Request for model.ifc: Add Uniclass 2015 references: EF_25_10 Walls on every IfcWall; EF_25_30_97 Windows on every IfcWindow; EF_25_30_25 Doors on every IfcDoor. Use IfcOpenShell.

First a look at what the model holds.

```python
import ifcopenshell

model = ifcopenshell.open("model.ifc")
print(model.schema)
print("classifications:", [c.Name for c in model.by_type("IfcClassification")])
for ifc_class in ("IfcDoor", "IfcRoof", "IfcStair", "IfcWall", "IfcWindow"):
    print(ifc_class, len(model.by_type(ifc_class)))
```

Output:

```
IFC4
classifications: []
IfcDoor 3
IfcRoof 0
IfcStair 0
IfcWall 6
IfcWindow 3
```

```python
import ifcopenshell
import ifcopenshell.api.classification

model = ifcopenshell.open("model.ifc")

system = ifcopenshell.api.classification.add_classification(model, classification="Uniclass 2015")

codes = {
    "IfcWall": ("EF_25_10", "Walls"),
    "IfcWindow": ("EF_25_30_97", "Windows"),
    "IfcDoor": ("EF_25_30_25", "Doors"),
}
for ifc_class, (code, name) in codes.items():
    products = model.by_type(ifc_class)
    ifcopenshell.api.classification.add_reference(
        model, products=products, classification=system, identification=code, name=name
    )
    print(code, len(products))

model.write("model-out.ifc")
```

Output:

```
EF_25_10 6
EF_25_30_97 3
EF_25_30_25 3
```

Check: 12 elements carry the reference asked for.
